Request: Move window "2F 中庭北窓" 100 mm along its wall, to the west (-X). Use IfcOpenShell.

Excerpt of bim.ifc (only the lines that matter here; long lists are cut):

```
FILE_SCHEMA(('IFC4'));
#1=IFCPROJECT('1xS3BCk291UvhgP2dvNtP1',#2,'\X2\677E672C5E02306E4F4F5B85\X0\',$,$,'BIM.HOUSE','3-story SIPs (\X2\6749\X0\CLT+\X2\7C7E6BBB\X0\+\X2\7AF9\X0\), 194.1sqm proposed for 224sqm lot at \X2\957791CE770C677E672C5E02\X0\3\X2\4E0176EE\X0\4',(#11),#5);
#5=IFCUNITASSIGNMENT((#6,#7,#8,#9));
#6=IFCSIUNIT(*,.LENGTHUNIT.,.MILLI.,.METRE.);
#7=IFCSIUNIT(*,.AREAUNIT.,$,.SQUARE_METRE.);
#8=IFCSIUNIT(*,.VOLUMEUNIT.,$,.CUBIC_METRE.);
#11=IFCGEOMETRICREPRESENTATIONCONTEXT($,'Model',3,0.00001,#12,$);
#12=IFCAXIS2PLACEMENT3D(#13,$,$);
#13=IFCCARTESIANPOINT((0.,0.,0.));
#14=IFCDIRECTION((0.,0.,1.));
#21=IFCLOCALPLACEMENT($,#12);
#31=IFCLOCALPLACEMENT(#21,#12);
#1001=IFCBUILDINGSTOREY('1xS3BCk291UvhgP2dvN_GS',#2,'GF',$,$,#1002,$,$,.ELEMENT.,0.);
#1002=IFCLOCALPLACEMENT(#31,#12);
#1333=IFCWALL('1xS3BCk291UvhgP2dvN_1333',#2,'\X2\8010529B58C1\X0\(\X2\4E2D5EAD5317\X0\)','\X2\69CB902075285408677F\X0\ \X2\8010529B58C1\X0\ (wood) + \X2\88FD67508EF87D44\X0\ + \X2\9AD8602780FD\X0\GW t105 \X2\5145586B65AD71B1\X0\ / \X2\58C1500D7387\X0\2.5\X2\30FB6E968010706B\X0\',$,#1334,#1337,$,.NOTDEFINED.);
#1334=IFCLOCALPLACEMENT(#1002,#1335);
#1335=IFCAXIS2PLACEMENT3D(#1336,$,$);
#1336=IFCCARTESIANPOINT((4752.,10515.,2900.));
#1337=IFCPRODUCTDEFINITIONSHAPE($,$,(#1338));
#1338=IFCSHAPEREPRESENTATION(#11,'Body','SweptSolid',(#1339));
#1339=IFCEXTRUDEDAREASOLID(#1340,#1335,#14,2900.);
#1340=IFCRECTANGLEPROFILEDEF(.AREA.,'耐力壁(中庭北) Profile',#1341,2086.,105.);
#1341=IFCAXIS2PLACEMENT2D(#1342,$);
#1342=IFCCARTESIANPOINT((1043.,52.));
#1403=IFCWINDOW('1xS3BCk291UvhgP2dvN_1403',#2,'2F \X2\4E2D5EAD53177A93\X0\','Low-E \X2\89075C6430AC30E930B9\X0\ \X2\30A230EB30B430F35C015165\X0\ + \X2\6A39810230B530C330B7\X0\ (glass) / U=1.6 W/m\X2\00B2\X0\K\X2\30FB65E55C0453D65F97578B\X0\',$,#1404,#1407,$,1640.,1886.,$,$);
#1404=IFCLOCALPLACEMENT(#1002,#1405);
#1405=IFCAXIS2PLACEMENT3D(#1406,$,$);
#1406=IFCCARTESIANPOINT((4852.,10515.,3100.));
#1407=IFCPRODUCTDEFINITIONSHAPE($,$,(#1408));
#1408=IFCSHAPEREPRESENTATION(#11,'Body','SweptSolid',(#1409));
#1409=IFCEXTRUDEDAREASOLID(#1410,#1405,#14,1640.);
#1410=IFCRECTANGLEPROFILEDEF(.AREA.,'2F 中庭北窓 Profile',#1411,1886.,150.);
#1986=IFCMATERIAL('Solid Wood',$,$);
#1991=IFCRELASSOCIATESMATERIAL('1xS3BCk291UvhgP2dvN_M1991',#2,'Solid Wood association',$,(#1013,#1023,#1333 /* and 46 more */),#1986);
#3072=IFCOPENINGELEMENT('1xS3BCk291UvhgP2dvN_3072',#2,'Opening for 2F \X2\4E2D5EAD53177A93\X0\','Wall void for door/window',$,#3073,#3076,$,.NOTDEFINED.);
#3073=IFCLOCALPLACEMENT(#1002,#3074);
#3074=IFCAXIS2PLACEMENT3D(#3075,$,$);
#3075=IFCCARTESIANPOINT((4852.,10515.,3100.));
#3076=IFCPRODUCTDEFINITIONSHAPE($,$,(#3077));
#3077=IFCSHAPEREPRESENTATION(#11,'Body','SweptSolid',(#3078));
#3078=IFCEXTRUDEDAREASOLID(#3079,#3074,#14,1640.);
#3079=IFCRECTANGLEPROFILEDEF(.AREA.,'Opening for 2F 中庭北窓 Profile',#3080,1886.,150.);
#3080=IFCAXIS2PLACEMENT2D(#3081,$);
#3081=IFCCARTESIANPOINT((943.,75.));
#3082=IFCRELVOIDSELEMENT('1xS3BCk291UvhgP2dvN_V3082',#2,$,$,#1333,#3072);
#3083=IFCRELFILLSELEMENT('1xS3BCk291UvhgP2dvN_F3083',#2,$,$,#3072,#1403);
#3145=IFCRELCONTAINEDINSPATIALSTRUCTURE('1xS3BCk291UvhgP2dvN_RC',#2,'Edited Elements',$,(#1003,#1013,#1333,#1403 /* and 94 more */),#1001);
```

```python
import ifcopenshell
import ifcopenshell.api.geometry
import ifcopenshell.util.placement

model = ifcopenshell.open("bim.ifc")

window = model.by_guid("1xS3BCk291UvhgP2dvN_1403")
opening = window.FillsVoids[0].RelatingOpeningElement
wall = opening.VoidsElements[0].RelatingBuildingElement

wall_matrix = ifcopenshell.util.placement.get_local_placement(wall.ObjectPlacement)
shift = wall_matrix[:3, 0] * -100.0
before = ifcopenshell.util.placement.get_local_placement(window.ObjectPlacement)[:3, 3].copy()

# The window is not placed relative to its opening, so move both.
for product in (opening, window):
    matrix = ifcopenshell.util.placement.get_local_placement(product.ObjectPlacement)
    matrix[:3, 3] += shift
    ifcopenshell.api.geometry.edit_object_placement(model, product=product, matrix=matrix, is_si=False)

after = ifcopenshell.util.placement.get_local_placement(window.ObjectPlacement)[:3, 3]
print("window moved by", (after - before).round(3) + 0.0)

model.write("bim_updated.ifc")
```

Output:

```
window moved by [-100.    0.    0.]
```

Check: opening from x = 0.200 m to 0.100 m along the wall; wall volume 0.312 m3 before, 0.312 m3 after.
